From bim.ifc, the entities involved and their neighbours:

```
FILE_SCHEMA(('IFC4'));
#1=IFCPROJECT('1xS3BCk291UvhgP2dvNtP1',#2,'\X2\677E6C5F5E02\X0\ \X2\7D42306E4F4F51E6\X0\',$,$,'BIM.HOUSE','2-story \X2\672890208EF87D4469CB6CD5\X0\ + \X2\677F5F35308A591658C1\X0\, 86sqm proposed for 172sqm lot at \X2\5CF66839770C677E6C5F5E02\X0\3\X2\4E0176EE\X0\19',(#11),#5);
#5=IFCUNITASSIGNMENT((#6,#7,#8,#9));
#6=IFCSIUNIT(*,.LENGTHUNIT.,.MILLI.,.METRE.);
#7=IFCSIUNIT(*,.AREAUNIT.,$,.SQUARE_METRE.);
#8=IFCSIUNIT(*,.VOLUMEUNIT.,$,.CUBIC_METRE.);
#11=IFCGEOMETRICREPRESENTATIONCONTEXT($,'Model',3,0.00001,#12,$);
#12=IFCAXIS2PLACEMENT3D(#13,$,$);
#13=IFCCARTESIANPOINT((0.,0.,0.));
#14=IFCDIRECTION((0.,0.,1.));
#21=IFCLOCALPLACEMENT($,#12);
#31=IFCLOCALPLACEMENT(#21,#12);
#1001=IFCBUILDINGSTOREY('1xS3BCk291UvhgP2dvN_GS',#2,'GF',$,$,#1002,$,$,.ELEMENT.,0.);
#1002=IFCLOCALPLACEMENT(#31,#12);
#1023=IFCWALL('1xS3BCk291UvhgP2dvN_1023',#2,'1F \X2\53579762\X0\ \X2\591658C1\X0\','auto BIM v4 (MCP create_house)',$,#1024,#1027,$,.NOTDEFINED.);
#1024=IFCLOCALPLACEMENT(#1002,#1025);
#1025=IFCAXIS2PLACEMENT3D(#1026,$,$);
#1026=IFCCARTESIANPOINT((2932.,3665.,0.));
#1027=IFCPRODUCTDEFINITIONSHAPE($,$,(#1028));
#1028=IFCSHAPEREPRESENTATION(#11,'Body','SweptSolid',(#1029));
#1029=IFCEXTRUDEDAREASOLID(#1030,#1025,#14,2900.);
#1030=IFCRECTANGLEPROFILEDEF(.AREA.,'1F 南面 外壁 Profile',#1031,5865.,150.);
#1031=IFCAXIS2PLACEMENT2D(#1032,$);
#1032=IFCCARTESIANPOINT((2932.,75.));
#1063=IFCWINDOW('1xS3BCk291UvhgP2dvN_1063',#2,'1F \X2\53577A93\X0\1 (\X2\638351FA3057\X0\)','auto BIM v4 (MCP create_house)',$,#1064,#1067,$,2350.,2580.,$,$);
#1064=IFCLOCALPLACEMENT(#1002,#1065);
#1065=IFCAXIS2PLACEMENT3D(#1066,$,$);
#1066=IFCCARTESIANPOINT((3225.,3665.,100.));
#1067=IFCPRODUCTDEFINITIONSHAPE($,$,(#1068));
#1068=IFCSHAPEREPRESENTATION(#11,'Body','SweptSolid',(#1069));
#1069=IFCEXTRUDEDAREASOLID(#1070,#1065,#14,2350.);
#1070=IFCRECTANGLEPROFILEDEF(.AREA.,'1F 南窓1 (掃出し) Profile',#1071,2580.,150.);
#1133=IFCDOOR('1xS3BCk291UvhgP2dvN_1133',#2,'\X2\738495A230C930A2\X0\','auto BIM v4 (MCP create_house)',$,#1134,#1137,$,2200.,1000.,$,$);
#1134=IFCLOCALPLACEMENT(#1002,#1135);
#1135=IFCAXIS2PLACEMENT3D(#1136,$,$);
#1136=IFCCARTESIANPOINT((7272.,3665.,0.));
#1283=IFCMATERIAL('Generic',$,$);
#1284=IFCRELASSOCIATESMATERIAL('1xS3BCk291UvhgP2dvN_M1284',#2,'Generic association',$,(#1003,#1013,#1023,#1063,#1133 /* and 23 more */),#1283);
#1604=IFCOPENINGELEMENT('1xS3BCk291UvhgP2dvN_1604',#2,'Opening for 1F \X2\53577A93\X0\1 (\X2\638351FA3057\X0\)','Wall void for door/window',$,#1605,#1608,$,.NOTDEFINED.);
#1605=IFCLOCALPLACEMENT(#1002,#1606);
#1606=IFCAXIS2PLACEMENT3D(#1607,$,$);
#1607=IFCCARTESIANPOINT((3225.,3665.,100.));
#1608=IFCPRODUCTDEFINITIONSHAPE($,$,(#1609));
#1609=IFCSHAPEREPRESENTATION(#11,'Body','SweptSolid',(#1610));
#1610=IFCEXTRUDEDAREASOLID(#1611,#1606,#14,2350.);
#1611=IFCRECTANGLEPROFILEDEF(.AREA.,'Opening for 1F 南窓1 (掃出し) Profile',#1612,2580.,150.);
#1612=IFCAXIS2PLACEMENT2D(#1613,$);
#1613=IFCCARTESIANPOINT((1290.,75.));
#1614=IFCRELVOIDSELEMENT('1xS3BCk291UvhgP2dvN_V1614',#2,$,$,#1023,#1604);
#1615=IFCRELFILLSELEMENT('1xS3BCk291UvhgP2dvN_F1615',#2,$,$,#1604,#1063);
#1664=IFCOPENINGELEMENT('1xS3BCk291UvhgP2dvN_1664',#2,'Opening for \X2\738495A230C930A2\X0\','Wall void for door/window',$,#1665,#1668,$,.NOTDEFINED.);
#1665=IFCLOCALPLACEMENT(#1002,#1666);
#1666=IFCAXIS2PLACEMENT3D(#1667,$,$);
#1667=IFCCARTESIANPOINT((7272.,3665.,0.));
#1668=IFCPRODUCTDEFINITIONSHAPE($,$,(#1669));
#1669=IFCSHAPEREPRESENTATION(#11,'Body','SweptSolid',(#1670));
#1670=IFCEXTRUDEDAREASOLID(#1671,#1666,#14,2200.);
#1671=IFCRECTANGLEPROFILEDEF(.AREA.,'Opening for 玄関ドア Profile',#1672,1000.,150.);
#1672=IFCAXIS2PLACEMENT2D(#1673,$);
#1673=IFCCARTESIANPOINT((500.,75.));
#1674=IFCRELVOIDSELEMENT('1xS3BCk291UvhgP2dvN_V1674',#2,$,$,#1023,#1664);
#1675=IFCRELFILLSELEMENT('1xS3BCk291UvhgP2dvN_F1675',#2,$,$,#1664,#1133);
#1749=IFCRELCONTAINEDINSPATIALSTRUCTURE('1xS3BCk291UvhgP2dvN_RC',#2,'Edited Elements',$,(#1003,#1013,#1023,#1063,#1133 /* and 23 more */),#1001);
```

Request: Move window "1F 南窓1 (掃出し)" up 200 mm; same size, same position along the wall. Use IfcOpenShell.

```python
import numpy as np
import ifcopenshell
import ifcopenshell.api.geometry
import ifcopenshell.util.placement
import ifcopenshell.util.unit

model = ifcopenshell.open("bim.ifc")
unit_scale = ifcopenshell.util.unit.calculate_unit_scale(model)

window = model.by_guid("1xS3BCk291UvhgP2dvN_1063")
opening = window.FillsVoids[0].RelatingOpeningElement
dz = 0.2 / unit_scale

shift = np.array([0.0, 0.0, dz])
# The window is not placed relative to its opening, so move both.
for product in (opening, window):
    matrix = ifcopenshell.util.placement.get_local_placement(product.ObjectPlacement)
    matrix[:3, 3] += shift
    ifcopenshell.api.geometry.edit_object_placement(model, product=product, matrix=matrix, is_si=False)

print(f"moved by {dz * unit_scale:+.3f} m")

model.write("bim_v2.ifc")
```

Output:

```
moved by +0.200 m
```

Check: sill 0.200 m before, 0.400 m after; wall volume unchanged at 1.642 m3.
